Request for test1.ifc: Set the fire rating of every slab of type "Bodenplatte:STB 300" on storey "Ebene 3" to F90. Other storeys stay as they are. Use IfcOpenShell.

First a look at what the model holds.

```python
import ifcopenshell
import ifcopenshell.util.element

model = ifcopenshell.open("test1.ifc")
print(model.schema)
storey = next(s for s in model.by_type("IfcBuildingStorey") if s.Name == "Ebene 3")
slabs = [e for e in ifcopenshell.util.element.get_decomposition(storey) if e.is_a("IfcSlab")]
seen = {}
for e in slabs:
    element_type = ifcopenshell.util.element.get_type(e)
    key = (element_type.Name if element_type != e and element_type else None, ifcopenshell.util.element.get_pset(e, "Pset_SlabCommon", "FireRating"))
    seen[key] = seen.get(key, 0) + 1
for (name, value), count in sorted(seen.items(), key=str):
    print(count, "x", name, "|", value)
```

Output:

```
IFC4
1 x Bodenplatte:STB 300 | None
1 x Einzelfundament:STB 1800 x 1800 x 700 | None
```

```python
import ifcopenshell
import ifcopenshell.api.pset
import ifcopenshell.util.element

model = ifcopenshell.open("test1.ifc")

storey = next(s for s in model.by_type("IfcBuildingStorey") if s.Name == "Ebene 3")
slabs = [e for e in ifcopenshell.util.element.get_decomposition(storey) if e.is_a("IfcSlab")]

count = 0
for e in slabs:
    element_type = ifcopenshell.util.element.get_type(e)
    if element_type in (None, e) or element_type.Name != "Bodenplatte:STB 300":
        continue
    # add_pset returns the element's existing set when there is one.
    pset = ifcopenshell.api.pset.add_pset(model, product=e, name="Pset_SlabCommon")
    ifcopenshell.api.pset.edit_pset(model, pset=pset, properties={"FireRating": "F90"})
    count += 1

print(count, "slabs updated")

model.write("test1_updated.ifc")
```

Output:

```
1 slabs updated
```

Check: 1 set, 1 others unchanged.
